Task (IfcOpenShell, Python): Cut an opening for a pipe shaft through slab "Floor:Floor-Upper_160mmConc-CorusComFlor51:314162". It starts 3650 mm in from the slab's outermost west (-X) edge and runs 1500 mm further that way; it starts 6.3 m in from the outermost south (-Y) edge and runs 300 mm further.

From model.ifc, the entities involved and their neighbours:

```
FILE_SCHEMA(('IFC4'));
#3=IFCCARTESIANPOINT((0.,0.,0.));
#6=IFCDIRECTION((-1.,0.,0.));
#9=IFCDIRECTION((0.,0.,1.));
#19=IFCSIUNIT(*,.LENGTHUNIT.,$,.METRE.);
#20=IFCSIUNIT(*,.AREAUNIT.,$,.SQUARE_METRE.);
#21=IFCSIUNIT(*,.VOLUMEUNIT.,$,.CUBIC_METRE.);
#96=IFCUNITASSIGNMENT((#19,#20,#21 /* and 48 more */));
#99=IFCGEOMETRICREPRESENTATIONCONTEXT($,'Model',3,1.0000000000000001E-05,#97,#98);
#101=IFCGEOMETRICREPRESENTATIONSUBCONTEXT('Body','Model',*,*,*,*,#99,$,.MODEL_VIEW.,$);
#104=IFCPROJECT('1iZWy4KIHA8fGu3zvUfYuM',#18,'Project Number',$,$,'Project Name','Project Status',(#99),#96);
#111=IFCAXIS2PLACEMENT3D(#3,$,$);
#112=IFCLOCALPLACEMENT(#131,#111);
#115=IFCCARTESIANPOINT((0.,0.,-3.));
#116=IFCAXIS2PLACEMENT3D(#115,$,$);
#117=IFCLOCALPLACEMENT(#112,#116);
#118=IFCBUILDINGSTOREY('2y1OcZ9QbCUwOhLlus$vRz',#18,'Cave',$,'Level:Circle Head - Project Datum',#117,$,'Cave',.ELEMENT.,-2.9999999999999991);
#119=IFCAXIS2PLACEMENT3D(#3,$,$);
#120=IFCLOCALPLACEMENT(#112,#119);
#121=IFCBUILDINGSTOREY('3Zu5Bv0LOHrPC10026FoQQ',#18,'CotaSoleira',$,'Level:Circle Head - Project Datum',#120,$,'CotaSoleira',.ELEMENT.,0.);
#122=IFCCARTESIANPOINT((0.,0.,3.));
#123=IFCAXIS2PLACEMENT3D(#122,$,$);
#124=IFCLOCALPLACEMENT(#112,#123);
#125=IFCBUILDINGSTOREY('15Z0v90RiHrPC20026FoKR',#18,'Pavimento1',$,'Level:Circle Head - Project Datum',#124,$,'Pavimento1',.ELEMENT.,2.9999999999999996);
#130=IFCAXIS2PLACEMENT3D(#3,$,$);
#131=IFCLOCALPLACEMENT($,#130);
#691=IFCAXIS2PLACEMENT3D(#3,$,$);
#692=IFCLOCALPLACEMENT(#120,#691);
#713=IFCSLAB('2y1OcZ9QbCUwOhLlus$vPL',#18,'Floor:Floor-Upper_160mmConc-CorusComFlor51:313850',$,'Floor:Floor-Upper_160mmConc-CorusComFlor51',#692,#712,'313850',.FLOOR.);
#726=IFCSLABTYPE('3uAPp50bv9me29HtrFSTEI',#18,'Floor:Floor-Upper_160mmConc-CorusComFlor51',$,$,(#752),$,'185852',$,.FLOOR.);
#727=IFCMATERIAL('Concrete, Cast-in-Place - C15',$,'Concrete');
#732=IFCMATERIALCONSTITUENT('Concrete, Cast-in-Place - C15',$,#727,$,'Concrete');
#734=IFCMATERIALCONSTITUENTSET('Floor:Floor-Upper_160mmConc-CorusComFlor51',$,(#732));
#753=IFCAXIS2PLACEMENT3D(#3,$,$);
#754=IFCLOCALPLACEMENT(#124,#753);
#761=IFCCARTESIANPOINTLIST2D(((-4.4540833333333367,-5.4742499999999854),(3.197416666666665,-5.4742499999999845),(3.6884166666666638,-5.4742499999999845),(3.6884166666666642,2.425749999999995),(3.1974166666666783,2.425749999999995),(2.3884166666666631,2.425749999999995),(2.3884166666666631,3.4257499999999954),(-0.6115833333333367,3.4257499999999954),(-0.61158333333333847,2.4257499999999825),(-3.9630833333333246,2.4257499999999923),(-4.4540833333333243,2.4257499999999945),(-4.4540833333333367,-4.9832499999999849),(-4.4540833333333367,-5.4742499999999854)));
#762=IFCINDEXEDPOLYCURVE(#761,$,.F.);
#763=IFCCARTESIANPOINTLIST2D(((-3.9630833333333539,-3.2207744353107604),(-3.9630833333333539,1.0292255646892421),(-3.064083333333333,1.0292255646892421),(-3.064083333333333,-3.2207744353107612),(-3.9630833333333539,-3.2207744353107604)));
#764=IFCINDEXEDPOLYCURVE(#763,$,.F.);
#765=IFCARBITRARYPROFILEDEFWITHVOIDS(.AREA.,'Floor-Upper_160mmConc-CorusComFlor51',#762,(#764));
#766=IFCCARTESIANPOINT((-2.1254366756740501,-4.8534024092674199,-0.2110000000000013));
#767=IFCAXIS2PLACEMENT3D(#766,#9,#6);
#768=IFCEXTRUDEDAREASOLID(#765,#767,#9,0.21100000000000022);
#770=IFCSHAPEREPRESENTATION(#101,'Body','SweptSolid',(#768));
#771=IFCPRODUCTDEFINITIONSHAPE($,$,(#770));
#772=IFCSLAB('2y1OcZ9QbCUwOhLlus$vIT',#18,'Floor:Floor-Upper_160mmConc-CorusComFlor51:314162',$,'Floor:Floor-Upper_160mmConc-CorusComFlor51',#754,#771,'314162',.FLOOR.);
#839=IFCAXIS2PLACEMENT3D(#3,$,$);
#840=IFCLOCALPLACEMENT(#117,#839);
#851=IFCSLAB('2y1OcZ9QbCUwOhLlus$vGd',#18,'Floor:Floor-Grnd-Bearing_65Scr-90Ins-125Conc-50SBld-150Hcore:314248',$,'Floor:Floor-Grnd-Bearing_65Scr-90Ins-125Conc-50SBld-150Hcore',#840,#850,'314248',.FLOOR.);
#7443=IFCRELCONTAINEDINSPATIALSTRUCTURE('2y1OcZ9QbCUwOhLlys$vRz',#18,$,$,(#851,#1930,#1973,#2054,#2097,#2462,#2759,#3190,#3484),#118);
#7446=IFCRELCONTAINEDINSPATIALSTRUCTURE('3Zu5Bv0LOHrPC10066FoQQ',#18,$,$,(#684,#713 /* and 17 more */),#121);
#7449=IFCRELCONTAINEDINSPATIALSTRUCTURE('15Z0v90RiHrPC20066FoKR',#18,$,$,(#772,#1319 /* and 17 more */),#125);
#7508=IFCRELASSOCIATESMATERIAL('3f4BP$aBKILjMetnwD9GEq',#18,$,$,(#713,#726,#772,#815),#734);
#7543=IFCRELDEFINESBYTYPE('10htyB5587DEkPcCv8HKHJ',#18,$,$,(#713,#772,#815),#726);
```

```python
import numpy as np
import ifcopenshell
import ifcopenshell.api.feature
import ifcopenshell.api.geometry
import ifcopenshell.api.root
import ifcopenshell.geom
import ifcopenshell.util.placement
import ifcopenshell.util.representation
import ifcopenshell.util.shape
import ifcopenshell.util.unit

model = ifcopenshell.open("model.ifc")
unit_scale = ifcopenshell.util.unit.calculate_unit_scale(model)
settings = ifcopenshell.geom.settings()


def volume(element):
    """Net volume in cubic metres, openings subtracted."""
    shape = ifcopenshell.geom.create_shape(settings, element)
    return ifcopenshell.util.shape.get_volume(shape.geometry)


slab = model.by_id(772)
before = volume(slab)

# Extent in the slab's own axes, in metres. The edges named are its -X and -Y sides.
slab_shape = ifcopenshell.geom.create_shape(settings, slab)
vertices = ifcopenshell.util.shape.get_vertices(slab_shape.geometry)
x_min, y_min, bottom = vertices.min(axis=0)
top = vertices[:, 2].max()

opening = ifcopenshell.api.root.create_entity(model, ifc_class="IfcOpeningElement", name="Pipe shaft opening", predefined_type="OPENING")
context = ifcopenshell.util.representation.get_context(model, "Model", "Body", "MODEL_VIEW")
width, depth = 1.5, 0.3
outline = [(0.0, 0.0), (width, 0.0), (width, depth), (0.0, depth), (0.0, 0.0)]
# Overshoot both faces by 50 mm so the cut is clean.
shape = ifcopenshell.api.geometry.add_slab_representation(
    model, context=context, depth=top - bottom + 0.1, polyline=outline
)
ifcopenshell.api.geometry.assign_representation(model, product=opening, representation=shape)

matrix = ifcopenshell.util.placement.get_local_placement(slab.ObjectPlacement)
matrix[:, 3] = matrix @ np.append(np.array([x_min + 3.65, y_min + 6.3, bottom - 0.05]) / unit_scale, 1.0)
ifcopenshell.api.geometry.edit_object_placement(model, product=opening, matrix=matrix, is_si=False)
ifcopenshell.api.feature.add_feature(model, feature=opening, element=slab)

after = volume(slab)

print(f"slab volume {before:.3f} -> {after:.3f} m3")

model.write("model_rev.ifc")
```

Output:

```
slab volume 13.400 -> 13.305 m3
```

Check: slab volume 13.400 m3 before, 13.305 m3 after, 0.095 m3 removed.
